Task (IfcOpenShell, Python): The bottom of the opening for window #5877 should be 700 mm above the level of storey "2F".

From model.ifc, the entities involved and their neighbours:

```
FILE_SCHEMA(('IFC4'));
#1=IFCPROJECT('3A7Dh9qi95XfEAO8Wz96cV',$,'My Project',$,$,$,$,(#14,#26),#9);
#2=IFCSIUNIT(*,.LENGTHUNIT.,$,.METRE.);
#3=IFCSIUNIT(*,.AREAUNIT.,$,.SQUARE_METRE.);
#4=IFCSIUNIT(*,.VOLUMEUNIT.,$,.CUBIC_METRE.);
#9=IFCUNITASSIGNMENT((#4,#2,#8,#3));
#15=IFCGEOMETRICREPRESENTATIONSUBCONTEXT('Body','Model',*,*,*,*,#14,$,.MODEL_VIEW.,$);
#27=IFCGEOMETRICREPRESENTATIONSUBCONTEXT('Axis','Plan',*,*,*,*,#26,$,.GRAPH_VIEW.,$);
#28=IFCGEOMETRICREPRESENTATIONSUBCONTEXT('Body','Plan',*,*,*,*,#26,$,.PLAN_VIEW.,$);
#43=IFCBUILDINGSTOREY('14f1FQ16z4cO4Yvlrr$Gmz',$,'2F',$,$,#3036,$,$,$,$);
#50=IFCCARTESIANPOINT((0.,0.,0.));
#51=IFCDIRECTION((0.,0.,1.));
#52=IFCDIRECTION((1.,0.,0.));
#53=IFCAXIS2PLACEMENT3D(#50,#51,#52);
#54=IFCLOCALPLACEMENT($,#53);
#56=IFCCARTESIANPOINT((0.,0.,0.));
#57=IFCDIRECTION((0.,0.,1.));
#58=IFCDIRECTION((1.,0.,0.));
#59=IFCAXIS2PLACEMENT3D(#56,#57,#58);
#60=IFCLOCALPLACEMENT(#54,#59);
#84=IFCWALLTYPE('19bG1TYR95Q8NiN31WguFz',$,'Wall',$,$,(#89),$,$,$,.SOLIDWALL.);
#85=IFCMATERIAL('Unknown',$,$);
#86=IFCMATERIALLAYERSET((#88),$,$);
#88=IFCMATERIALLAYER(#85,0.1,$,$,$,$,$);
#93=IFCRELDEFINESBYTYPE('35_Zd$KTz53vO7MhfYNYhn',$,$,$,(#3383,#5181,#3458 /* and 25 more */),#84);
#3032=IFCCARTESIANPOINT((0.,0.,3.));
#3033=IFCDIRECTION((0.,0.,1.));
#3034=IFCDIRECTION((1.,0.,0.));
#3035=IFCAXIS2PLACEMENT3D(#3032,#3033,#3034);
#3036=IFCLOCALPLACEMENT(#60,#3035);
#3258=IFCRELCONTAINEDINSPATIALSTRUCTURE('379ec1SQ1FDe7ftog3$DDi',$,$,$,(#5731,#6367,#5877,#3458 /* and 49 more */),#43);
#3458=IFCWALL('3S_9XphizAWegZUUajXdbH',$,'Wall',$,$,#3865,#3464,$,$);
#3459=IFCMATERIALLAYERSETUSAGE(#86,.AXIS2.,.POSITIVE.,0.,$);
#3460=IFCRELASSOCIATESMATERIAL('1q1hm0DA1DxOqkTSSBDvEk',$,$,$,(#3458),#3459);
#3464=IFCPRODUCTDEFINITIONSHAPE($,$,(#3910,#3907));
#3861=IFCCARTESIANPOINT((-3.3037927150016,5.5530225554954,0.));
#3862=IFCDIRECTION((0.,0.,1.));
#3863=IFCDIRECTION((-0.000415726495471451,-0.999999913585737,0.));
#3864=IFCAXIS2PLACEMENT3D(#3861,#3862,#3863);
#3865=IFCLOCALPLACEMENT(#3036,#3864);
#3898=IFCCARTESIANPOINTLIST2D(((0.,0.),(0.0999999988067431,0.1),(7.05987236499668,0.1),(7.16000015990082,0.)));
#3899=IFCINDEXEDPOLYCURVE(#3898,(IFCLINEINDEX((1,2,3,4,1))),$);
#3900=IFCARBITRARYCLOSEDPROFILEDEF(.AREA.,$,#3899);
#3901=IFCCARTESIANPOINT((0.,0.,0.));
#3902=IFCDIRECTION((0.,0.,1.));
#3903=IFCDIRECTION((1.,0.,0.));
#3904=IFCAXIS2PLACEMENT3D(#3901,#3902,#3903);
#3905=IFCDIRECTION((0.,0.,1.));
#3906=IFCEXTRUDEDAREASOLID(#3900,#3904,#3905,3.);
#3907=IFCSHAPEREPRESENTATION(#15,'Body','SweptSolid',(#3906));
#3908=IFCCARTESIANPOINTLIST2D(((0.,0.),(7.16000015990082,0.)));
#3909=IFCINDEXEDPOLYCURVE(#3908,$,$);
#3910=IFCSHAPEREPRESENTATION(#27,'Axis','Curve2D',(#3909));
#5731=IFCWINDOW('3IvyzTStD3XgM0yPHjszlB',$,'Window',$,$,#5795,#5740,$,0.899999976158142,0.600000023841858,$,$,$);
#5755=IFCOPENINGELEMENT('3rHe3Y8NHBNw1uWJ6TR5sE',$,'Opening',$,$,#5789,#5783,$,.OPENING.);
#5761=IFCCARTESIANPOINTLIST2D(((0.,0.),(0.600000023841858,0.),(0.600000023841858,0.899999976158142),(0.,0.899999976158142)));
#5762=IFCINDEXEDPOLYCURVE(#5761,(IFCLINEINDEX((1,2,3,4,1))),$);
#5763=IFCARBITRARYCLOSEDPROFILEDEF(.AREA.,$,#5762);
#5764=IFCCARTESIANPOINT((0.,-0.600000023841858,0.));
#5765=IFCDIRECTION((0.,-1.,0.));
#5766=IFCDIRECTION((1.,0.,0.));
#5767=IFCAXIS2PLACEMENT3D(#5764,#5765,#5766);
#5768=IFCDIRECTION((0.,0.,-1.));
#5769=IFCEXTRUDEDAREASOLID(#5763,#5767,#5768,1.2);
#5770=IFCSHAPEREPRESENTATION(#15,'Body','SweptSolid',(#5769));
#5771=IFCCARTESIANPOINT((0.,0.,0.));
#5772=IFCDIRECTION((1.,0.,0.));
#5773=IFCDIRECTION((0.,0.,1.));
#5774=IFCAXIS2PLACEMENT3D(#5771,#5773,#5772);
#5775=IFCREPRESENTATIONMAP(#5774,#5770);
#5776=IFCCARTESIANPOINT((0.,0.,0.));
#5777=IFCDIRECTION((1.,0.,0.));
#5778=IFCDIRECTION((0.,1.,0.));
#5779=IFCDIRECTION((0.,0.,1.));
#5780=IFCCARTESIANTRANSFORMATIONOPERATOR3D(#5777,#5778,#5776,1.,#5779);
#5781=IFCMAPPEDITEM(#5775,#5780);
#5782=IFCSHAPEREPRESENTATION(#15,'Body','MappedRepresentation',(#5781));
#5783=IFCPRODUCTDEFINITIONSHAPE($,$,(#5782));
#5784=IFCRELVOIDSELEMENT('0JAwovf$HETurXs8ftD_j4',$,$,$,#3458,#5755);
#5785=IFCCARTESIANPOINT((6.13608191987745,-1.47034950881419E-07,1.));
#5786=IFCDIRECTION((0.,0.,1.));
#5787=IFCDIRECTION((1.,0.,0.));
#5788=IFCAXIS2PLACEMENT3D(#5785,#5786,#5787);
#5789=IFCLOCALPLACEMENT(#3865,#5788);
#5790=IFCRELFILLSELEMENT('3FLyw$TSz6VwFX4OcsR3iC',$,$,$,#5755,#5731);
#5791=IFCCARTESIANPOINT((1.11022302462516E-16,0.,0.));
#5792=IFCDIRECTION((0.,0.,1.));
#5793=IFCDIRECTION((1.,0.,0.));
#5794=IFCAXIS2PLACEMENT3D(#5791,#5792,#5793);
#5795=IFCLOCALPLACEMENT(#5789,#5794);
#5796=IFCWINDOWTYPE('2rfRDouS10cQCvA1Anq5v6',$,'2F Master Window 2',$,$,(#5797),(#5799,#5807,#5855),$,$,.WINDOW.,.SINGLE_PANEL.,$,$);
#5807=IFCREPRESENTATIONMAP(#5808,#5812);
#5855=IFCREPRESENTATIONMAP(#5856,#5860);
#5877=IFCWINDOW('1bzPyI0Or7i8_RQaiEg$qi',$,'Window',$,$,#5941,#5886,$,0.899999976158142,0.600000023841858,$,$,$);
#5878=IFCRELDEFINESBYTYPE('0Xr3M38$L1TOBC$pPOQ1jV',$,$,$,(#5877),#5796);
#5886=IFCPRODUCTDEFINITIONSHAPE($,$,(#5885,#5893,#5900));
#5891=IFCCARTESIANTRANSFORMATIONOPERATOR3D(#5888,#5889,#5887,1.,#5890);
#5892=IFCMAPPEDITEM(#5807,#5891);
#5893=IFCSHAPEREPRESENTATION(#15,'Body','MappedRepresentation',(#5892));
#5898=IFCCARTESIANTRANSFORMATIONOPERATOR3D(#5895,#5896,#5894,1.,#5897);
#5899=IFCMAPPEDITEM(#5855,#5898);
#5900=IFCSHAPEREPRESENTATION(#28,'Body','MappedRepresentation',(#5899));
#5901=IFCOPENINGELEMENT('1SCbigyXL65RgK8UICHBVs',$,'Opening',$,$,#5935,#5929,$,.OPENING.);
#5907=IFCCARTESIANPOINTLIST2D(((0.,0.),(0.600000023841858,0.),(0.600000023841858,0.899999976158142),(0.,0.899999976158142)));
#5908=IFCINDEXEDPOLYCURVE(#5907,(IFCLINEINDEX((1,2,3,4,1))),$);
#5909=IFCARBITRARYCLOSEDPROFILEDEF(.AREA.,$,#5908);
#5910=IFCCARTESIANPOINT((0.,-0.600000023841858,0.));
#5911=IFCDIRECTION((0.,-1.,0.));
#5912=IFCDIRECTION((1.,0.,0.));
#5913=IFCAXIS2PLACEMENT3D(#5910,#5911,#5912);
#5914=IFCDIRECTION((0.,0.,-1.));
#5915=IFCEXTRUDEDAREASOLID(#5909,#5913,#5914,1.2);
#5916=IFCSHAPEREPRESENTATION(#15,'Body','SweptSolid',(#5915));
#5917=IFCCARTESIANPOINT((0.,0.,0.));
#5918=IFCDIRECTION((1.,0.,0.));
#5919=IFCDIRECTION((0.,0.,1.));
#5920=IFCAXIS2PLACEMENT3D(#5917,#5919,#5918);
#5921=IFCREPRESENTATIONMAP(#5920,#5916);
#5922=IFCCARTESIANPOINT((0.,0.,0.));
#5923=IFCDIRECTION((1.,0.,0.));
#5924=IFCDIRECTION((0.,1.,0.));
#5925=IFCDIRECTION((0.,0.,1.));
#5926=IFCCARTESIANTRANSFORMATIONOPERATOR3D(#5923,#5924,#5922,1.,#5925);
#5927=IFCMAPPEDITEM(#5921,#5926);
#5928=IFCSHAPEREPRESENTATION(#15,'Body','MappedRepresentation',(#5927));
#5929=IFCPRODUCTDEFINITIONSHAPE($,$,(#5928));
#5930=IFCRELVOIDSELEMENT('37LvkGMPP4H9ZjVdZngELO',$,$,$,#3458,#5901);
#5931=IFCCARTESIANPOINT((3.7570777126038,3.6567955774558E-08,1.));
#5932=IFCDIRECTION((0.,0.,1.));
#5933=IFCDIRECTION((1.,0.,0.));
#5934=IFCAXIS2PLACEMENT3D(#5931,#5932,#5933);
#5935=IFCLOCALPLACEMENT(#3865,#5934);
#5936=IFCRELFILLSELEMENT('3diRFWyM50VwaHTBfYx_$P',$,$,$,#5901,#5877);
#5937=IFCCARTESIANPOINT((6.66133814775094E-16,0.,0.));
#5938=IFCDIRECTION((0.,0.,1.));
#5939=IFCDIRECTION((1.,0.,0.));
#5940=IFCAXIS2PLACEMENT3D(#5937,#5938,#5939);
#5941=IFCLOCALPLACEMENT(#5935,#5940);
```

```python
import numpy as np
import ifcopenshell
import ifcopenshell.api.geometry
import ifcopenshell.geom
import ifcopenshell.util.element
import ifcopenshell.util.placement
import ifcopenshell.util.shape
import ifcopenshell.util.unit

model = ifcopenshell.open("model.ifc")
unit_scale = ifcopenshell.util.unit.calculate_unit_scale(model)

window = model.by_guid("1bzPyI0Or7i8_RQaiEg$qi")
opening = window.FillsVoids[0].RelatingOpeningElement
storey = ifcopenshell.util.element.get_container(window, ifc_class="IfcBuildingStorey")
level = ifcopenshell.util.placement.get_local_placement(storey.ObjectPlacement)[2, 3]

# The opening's origin need not be at the sill, so measure its lowest point.
shape = ifcopenshell.geom.create_shape(ifcopenshell.geom.settings(), opening)
bottom = ifcopenshell.util.shape.get_shape_bottom_elevation(shape, shape.geometry) / unit_scale
dz = level + 0.7 - bottom

shift = np.array([0.0, 0.0, dz])
# The window is placed relative to its opening, so it follows when the opening moves.
matrix = ifcopenshell.util.placement.get_local_placement(opening.ObjectPlacement)
matrix[:3, 3] += shift
ifcopenshell.api.geometry.edit_object_placement(
    model, product=opening, matrix=matrix, is_si=False, should_transform_children=True
)

print(f"moved by {dz * unit_scale:+.3f} m")

model.write("model_v2.ifc")
```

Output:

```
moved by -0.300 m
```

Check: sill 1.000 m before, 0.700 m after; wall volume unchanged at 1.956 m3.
